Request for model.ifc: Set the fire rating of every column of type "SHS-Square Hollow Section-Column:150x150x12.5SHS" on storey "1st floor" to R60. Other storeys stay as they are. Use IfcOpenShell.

First a look at what the model holds.

```python
import ifcopenshell
import ifcopenshell.util.element

model = ifcopenshell.open("model.ifc")
print(model.schema)
storey = next(s for s in model.by_type("IfcBuildingStorey") if s.Name == "1st floor")
columns = [e for e in ifcopenshell.util.element.get_decomposition(storey) if e.is_a("IfcColumn")]
seen = {}
for e in columns:
    element_type = ifcopenshell.util.element.get_type(e)
    key = (element_type.Name if element_type != e and element_type else None, ifcopenshell.util.element.get_pset(e, "Pset_ColumnCommon", "FireRating"))
    seen[key] = seen.get(key, 0) + 1
for (name, value), count in sorted(seen.items(), key=str):
    print(count, "x", name, "|", value)
```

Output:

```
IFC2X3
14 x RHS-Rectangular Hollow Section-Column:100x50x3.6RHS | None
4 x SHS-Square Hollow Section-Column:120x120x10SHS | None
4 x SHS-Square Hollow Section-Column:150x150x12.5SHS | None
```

```python
import ifcopenshell
import ifcopenshell.api.pset
import ifcopenshell.util.element

model = ifcopenshell.open("model.ifc")

storey = next(s for s in model.by_type("IfcBuildingStorey") if s.Name == "1st floor")
columns = [e for e in ifcopenshell.util.element.get_decomposition(storey) if e.is_a("IfcColumn")]

count = 0
for e in columns:
    element_type = ifcopenshell.util.element.get_type(e)
    if element_type in (None, e) or element_type.Name != "SHS-Square Hollow Section-Column:150x150x12.5SHS":
        continue
    # add_pset returns the element's existing set when there is one.
    pset = ifcopenshell.api.pset.add_pset(model, product=e, name="Pset_ColumnCommon")
    ifcopenshell.api.pset.edit_pset(model, pset=pset, properties={"FireRating": "R60"})
    count += 1

print(count, "columns updated")

model.write("model-out.ifc")
```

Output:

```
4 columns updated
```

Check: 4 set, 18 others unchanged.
